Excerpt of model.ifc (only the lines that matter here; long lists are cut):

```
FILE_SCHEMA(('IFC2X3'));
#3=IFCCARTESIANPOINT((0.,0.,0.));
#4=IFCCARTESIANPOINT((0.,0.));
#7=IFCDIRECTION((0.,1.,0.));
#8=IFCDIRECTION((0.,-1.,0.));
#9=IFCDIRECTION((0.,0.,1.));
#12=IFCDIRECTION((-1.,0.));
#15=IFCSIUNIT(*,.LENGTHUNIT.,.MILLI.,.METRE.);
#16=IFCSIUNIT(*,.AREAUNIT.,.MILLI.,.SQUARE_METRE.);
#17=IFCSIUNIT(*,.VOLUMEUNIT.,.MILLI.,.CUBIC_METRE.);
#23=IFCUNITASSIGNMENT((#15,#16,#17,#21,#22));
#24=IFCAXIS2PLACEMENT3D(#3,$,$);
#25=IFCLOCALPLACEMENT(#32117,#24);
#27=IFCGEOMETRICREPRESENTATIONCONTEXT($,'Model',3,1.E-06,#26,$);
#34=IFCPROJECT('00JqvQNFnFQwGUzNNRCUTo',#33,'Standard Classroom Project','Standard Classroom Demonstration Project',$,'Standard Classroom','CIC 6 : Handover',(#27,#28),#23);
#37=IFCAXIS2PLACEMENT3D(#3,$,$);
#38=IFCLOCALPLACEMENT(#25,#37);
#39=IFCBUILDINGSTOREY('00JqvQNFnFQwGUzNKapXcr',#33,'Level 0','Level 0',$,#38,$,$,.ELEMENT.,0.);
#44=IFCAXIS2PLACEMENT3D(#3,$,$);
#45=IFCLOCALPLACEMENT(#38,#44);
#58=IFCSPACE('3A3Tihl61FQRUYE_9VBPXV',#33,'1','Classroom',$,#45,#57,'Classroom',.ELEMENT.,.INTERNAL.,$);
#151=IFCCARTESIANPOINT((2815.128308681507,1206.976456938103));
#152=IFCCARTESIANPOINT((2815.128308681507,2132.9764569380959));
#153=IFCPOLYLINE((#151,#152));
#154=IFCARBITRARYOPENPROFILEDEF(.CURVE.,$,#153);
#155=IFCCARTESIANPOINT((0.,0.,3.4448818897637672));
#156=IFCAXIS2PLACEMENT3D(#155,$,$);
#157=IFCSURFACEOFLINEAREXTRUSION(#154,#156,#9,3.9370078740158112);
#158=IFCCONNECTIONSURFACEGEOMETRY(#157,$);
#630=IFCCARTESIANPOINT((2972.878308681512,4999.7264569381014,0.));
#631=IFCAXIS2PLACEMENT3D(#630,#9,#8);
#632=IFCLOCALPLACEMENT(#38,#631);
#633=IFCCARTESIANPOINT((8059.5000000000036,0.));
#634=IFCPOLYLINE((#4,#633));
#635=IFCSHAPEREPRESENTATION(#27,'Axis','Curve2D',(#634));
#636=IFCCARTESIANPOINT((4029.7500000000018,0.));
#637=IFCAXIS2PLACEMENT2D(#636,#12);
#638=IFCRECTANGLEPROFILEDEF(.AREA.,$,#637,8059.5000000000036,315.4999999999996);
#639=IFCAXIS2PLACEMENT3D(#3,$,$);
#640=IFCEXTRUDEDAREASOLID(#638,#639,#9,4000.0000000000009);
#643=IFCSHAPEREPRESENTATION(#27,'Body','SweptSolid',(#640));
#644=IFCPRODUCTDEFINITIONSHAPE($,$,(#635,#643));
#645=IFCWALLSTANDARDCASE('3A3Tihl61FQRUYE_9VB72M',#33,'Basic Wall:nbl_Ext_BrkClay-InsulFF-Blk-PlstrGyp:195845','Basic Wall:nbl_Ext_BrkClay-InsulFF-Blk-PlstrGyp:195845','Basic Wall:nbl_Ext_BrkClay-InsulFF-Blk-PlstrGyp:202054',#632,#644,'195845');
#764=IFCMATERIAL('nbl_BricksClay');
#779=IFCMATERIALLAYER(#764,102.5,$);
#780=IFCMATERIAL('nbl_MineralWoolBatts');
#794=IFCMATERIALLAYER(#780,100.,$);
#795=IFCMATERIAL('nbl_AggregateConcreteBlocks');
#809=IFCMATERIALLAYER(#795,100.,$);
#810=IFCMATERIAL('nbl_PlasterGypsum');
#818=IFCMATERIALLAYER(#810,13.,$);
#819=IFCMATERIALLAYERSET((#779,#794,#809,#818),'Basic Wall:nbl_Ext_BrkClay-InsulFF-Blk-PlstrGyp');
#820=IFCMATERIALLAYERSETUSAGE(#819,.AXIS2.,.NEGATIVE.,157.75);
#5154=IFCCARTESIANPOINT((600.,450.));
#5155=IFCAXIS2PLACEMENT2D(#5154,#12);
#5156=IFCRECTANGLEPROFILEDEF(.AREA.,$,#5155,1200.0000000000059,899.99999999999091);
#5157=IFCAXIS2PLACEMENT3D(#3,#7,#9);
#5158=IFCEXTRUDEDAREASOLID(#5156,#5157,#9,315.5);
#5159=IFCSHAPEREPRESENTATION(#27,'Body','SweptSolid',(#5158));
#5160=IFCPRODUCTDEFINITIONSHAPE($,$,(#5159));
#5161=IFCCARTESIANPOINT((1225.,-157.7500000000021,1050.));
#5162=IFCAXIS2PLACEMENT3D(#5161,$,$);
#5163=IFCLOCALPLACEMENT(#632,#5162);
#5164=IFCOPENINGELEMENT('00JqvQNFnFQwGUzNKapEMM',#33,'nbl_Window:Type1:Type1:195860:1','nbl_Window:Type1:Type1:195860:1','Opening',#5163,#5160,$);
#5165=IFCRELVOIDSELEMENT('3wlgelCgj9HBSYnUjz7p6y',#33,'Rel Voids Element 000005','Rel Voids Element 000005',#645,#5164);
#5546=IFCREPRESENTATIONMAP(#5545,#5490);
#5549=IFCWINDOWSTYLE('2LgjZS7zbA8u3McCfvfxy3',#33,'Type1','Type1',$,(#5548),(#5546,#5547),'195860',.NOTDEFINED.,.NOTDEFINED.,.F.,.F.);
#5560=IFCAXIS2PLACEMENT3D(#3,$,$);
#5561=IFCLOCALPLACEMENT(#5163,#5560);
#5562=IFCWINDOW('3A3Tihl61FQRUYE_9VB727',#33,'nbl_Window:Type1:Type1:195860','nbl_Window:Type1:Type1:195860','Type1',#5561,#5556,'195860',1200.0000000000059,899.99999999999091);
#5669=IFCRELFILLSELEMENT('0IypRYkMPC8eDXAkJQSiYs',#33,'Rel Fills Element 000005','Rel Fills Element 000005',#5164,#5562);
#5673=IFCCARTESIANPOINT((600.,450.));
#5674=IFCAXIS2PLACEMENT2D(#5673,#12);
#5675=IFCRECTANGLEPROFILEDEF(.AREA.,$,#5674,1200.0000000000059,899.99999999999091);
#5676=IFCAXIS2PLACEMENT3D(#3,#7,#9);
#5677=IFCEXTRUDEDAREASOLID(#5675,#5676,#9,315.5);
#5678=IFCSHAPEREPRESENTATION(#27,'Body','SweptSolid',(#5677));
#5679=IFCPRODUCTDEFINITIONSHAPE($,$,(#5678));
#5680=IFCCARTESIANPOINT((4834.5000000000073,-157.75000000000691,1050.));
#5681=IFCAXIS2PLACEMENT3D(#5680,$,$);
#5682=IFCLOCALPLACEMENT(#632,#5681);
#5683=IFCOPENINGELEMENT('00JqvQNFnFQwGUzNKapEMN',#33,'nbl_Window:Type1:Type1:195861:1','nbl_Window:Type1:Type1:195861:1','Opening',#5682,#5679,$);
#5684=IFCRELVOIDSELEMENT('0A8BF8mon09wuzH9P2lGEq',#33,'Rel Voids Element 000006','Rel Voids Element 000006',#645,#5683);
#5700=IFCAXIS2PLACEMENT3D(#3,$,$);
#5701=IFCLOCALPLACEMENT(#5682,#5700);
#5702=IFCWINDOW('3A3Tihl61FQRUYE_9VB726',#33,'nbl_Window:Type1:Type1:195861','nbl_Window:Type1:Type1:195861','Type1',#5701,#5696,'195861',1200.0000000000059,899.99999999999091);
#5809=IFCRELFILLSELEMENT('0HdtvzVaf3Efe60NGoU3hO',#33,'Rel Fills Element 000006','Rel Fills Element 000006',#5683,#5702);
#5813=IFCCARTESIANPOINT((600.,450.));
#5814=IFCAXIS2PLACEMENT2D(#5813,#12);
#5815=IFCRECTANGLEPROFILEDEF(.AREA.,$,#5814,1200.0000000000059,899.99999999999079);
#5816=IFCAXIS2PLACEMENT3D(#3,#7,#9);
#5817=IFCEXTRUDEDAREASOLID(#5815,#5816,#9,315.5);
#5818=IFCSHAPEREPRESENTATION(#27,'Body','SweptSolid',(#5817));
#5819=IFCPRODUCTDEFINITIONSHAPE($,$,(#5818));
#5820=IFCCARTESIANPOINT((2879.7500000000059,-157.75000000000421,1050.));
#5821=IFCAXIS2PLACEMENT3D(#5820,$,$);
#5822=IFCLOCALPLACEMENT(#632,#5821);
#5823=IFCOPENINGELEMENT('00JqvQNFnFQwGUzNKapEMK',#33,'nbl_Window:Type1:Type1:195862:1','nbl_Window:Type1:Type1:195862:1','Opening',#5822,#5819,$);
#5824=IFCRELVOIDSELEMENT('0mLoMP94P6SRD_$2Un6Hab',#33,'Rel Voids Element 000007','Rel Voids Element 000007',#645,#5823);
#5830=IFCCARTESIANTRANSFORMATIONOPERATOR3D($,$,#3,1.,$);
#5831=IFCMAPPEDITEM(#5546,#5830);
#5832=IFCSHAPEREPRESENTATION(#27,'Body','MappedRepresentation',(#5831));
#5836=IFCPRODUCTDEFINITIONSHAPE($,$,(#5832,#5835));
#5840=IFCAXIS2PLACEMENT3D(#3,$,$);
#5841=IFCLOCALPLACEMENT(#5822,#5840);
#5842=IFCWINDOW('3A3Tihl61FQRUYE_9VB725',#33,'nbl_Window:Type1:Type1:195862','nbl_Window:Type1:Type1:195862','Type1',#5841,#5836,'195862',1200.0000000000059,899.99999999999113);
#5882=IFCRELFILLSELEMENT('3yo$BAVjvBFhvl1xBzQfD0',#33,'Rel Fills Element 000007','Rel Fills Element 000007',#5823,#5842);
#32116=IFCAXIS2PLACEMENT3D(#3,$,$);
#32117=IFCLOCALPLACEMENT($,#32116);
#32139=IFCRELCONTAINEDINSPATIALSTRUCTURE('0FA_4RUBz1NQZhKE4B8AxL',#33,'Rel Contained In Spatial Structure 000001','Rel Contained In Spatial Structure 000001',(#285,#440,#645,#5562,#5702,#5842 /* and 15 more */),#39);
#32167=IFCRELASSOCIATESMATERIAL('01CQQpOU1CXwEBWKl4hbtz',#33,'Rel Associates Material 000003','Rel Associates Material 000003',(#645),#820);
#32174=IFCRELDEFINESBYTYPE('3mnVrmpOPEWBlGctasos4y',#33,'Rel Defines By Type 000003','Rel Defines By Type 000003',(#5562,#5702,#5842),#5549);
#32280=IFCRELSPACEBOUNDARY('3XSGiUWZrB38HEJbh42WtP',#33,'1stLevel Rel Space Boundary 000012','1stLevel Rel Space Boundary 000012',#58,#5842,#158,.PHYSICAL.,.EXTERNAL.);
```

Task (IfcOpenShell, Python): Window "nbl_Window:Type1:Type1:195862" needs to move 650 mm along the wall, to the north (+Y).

```python
import numpy as np
import ifcopenshell
import ifcopenshell.api.geometry
import ifcopenshell.util.placement
import ifcopenshell.util.unit

model = ifcopenshell.open("model.ifc")
unit_scale = ifcopenshell.util.unit.calculate_unit_scale(model)

window = model.by_guid("3A3Tihl61FQRUYE_9VB725")
opening = window.FillsVoids[0].RelatingOpeningElement
wall = opening.VoidsElements[0].RelatingBuildingElement

wall_matrix = ifcopenshell.util.placement.get_local_placement(wall.ObjectPlacement)
shift = wall_matrix[:3, 0] * -0.65 / unit_scale
before = ifcopenshell.util.placement.get_local_placement(window.ObjectPlacement)[:3, 3].copy()

# The window is placed relative to its opening, so it follows when the opening moves.
matrix = ifcopenshell.util.placement.get_local_placement(opening.ObjectPlacement)
matrix[:3, 3] += shift
ifcopenshell.api.geometry.edit_object_placement(
    model, product=opening, matrix=matrix, is_si=False, should_transform_children=True
)

# Space boundary surfaces are stored in each space's coordinates; move them too.
for rel in window.ProvidesBoundaries:
    if not rel.ConnectionGeometry:
        continue
    surface = rel.ConnectionGeometry.SurfaceOnRelatingElement
    space_matrix = ifcopenshell.util.placement.get_local_placement(rel.RelatingSpace.ObjectPlacement)
    point = np.array(surface.Position.Location.Coordinates) + space_matrix[:3, :3].T @ shift
    surface.Position = model.createIfcAxis2Placement3D(
        model.createIfcCartesianPoint(point.tolist()), surface.Position.Axis, surface.Position.RefDirection
    )

after = ifcopenshell.util.placement.get_local_placement(window.ObjectPlacement)[:3, 3]
print("window moved by", (after - before).round(3) + 0.0)

model.write("model_v2.ifc")
```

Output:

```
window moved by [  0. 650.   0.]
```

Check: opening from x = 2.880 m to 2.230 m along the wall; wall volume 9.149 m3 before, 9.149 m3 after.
